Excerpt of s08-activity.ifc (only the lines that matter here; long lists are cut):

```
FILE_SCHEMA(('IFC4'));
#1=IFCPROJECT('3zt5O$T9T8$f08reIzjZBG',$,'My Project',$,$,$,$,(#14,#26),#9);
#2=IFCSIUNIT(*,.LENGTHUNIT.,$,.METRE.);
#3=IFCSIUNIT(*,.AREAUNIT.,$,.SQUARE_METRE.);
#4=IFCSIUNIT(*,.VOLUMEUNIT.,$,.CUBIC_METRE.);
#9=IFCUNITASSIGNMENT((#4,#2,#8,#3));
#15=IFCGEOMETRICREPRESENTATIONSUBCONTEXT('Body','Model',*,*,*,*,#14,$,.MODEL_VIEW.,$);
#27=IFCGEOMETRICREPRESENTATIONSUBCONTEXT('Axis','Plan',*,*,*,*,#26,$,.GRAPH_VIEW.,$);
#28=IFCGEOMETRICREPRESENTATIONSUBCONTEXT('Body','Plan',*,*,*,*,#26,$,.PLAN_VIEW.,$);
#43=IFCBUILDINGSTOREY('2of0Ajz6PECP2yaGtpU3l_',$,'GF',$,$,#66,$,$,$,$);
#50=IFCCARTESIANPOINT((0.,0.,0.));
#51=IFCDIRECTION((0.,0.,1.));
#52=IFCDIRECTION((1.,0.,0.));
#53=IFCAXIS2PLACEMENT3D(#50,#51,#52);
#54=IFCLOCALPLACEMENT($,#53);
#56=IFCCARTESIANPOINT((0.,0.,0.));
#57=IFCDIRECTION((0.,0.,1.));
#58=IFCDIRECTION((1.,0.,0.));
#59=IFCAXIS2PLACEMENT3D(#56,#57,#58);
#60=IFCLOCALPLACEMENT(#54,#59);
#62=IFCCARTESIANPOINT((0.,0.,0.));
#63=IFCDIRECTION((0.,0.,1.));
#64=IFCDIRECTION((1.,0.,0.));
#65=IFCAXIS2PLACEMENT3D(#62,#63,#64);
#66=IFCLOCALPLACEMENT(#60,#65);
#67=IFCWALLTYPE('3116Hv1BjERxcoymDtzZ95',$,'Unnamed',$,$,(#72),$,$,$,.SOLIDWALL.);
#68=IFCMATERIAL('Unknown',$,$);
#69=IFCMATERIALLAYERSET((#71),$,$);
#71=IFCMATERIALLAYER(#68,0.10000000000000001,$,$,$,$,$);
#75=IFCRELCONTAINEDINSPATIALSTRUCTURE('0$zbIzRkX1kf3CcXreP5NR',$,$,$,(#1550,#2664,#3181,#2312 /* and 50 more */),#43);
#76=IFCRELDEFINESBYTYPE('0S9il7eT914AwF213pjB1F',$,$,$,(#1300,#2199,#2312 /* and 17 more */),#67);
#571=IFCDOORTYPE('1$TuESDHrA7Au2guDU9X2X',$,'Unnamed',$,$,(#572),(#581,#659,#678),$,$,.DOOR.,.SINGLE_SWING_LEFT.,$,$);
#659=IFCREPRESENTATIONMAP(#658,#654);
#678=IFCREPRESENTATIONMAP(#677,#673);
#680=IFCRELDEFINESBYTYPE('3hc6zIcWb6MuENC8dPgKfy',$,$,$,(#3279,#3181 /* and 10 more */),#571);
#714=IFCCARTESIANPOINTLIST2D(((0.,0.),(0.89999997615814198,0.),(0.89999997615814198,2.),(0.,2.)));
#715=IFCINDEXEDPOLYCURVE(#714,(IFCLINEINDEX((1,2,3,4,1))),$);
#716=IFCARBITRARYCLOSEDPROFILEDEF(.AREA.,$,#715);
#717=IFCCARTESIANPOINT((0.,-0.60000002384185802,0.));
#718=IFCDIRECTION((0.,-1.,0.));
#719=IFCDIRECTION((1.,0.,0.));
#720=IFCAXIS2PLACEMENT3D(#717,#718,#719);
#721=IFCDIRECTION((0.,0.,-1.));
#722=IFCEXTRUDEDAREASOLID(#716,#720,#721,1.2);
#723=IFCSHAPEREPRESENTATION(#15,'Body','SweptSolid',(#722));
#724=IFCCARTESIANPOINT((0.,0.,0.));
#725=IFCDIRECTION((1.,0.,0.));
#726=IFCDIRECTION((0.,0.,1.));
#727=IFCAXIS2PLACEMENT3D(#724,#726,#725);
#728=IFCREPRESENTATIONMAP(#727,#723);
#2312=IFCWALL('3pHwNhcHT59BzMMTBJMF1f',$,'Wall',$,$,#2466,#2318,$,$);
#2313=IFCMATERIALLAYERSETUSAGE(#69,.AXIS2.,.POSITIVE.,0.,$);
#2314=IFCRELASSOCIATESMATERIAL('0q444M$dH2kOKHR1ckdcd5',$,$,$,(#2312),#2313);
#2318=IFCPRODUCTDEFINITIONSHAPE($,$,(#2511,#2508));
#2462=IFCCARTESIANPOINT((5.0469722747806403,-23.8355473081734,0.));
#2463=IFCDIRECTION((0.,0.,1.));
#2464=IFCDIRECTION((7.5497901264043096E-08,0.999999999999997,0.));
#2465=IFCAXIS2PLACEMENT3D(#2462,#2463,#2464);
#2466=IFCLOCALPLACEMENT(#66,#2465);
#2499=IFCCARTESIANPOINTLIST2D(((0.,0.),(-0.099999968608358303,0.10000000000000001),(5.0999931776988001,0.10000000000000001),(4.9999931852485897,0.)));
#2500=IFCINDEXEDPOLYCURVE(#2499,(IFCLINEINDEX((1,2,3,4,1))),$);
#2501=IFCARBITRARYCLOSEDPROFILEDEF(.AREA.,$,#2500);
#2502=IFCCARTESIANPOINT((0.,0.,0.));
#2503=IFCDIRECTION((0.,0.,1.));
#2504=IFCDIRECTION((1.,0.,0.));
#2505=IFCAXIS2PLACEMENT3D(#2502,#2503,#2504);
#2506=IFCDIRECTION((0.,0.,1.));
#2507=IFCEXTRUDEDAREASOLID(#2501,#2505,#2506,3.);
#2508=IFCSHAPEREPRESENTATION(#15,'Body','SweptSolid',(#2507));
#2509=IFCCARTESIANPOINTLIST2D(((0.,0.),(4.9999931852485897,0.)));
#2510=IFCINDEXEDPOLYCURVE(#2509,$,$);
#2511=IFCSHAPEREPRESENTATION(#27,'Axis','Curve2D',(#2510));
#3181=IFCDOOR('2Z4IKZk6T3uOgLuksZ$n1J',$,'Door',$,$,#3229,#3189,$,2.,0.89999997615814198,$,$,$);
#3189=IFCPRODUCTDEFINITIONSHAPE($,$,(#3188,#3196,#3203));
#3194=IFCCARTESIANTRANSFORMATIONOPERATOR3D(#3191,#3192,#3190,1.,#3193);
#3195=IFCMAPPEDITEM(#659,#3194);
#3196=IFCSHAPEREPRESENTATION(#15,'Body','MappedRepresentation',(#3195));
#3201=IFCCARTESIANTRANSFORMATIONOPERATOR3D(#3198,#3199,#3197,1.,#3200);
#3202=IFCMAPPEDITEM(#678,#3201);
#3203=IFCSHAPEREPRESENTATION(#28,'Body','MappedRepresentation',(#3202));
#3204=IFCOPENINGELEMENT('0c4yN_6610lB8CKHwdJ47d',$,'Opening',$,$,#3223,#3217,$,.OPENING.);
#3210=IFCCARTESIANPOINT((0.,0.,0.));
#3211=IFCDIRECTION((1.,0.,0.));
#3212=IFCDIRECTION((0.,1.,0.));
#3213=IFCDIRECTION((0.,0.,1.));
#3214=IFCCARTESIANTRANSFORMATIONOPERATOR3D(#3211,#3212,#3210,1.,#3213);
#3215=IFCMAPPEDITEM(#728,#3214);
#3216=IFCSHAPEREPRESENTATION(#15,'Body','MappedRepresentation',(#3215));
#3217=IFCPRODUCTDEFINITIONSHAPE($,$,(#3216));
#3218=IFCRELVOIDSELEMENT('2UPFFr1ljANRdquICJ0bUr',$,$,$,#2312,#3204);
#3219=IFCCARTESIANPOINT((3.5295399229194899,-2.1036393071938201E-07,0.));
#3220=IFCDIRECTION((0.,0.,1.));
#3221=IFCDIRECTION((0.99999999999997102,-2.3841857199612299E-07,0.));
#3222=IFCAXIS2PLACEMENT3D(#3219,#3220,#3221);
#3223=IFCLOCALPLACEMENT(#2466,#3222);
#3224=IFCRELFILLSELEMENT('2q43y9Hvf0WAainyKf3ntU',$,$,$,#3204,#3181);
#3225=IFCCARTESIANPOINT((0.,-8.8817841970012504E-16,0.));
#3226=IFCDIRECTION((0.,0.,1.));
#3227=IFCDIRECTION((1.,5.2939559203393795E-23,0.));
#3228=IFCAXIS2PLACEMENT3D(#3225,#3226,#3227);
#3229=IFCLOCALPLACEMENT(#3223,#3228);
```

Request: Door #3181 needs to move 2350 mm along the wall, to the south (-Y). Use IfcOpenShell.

```python
import ifcopenshell
import ifcopenshell.api.geometry
import ifcopenshell.util.placement
import ifcopenshell.util.unit

model = ifcopenshell.open("s08-activity.ifc")
unit_scale = ifcopenshell.util.unit.calculate_unit_scale(model)

door = model.by_guid("2Z4IKZk6T3uOgLuksZ$n1J")
opening = door.FillsVoids[0].RelatingOpeningElement
wall = opening.VoidsElements[0].RelatingBuildingElement

wall_matrix = ifcopenshell.util.placement.get_local_placement(wall.ObjectPlacement)
shift = wall_matrix[:3, 0] * -2.35 / unit_scale
before = ifcopenshell.util.placement.get_local_placement(door.ObjectPlacement)[:3, 3].copy()

# The door is placed relative to its opening, so it follows when the opening moves.
matrix = ifcopenshell.util.placement.get_local_placement(opening.ObjectPlacement)
matrix[:3, 3] += shift
ifcopenshell.api.geometry.edit_object_placement(
    model, product=opening, matrix=matrix, is_si=False, should_transform_children=True
)

after = ifcopenshell.util.placement.get_local_placement(door.ObjectPlacement)[:3, 3]
print("door moved by", (after - before).round(3) + 0.0)

model.write("s08-activity-out.ifc")
```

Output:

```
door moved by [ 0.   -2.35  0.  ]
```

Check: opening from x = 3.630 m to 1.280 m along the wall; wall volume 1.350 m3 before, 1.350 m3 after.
